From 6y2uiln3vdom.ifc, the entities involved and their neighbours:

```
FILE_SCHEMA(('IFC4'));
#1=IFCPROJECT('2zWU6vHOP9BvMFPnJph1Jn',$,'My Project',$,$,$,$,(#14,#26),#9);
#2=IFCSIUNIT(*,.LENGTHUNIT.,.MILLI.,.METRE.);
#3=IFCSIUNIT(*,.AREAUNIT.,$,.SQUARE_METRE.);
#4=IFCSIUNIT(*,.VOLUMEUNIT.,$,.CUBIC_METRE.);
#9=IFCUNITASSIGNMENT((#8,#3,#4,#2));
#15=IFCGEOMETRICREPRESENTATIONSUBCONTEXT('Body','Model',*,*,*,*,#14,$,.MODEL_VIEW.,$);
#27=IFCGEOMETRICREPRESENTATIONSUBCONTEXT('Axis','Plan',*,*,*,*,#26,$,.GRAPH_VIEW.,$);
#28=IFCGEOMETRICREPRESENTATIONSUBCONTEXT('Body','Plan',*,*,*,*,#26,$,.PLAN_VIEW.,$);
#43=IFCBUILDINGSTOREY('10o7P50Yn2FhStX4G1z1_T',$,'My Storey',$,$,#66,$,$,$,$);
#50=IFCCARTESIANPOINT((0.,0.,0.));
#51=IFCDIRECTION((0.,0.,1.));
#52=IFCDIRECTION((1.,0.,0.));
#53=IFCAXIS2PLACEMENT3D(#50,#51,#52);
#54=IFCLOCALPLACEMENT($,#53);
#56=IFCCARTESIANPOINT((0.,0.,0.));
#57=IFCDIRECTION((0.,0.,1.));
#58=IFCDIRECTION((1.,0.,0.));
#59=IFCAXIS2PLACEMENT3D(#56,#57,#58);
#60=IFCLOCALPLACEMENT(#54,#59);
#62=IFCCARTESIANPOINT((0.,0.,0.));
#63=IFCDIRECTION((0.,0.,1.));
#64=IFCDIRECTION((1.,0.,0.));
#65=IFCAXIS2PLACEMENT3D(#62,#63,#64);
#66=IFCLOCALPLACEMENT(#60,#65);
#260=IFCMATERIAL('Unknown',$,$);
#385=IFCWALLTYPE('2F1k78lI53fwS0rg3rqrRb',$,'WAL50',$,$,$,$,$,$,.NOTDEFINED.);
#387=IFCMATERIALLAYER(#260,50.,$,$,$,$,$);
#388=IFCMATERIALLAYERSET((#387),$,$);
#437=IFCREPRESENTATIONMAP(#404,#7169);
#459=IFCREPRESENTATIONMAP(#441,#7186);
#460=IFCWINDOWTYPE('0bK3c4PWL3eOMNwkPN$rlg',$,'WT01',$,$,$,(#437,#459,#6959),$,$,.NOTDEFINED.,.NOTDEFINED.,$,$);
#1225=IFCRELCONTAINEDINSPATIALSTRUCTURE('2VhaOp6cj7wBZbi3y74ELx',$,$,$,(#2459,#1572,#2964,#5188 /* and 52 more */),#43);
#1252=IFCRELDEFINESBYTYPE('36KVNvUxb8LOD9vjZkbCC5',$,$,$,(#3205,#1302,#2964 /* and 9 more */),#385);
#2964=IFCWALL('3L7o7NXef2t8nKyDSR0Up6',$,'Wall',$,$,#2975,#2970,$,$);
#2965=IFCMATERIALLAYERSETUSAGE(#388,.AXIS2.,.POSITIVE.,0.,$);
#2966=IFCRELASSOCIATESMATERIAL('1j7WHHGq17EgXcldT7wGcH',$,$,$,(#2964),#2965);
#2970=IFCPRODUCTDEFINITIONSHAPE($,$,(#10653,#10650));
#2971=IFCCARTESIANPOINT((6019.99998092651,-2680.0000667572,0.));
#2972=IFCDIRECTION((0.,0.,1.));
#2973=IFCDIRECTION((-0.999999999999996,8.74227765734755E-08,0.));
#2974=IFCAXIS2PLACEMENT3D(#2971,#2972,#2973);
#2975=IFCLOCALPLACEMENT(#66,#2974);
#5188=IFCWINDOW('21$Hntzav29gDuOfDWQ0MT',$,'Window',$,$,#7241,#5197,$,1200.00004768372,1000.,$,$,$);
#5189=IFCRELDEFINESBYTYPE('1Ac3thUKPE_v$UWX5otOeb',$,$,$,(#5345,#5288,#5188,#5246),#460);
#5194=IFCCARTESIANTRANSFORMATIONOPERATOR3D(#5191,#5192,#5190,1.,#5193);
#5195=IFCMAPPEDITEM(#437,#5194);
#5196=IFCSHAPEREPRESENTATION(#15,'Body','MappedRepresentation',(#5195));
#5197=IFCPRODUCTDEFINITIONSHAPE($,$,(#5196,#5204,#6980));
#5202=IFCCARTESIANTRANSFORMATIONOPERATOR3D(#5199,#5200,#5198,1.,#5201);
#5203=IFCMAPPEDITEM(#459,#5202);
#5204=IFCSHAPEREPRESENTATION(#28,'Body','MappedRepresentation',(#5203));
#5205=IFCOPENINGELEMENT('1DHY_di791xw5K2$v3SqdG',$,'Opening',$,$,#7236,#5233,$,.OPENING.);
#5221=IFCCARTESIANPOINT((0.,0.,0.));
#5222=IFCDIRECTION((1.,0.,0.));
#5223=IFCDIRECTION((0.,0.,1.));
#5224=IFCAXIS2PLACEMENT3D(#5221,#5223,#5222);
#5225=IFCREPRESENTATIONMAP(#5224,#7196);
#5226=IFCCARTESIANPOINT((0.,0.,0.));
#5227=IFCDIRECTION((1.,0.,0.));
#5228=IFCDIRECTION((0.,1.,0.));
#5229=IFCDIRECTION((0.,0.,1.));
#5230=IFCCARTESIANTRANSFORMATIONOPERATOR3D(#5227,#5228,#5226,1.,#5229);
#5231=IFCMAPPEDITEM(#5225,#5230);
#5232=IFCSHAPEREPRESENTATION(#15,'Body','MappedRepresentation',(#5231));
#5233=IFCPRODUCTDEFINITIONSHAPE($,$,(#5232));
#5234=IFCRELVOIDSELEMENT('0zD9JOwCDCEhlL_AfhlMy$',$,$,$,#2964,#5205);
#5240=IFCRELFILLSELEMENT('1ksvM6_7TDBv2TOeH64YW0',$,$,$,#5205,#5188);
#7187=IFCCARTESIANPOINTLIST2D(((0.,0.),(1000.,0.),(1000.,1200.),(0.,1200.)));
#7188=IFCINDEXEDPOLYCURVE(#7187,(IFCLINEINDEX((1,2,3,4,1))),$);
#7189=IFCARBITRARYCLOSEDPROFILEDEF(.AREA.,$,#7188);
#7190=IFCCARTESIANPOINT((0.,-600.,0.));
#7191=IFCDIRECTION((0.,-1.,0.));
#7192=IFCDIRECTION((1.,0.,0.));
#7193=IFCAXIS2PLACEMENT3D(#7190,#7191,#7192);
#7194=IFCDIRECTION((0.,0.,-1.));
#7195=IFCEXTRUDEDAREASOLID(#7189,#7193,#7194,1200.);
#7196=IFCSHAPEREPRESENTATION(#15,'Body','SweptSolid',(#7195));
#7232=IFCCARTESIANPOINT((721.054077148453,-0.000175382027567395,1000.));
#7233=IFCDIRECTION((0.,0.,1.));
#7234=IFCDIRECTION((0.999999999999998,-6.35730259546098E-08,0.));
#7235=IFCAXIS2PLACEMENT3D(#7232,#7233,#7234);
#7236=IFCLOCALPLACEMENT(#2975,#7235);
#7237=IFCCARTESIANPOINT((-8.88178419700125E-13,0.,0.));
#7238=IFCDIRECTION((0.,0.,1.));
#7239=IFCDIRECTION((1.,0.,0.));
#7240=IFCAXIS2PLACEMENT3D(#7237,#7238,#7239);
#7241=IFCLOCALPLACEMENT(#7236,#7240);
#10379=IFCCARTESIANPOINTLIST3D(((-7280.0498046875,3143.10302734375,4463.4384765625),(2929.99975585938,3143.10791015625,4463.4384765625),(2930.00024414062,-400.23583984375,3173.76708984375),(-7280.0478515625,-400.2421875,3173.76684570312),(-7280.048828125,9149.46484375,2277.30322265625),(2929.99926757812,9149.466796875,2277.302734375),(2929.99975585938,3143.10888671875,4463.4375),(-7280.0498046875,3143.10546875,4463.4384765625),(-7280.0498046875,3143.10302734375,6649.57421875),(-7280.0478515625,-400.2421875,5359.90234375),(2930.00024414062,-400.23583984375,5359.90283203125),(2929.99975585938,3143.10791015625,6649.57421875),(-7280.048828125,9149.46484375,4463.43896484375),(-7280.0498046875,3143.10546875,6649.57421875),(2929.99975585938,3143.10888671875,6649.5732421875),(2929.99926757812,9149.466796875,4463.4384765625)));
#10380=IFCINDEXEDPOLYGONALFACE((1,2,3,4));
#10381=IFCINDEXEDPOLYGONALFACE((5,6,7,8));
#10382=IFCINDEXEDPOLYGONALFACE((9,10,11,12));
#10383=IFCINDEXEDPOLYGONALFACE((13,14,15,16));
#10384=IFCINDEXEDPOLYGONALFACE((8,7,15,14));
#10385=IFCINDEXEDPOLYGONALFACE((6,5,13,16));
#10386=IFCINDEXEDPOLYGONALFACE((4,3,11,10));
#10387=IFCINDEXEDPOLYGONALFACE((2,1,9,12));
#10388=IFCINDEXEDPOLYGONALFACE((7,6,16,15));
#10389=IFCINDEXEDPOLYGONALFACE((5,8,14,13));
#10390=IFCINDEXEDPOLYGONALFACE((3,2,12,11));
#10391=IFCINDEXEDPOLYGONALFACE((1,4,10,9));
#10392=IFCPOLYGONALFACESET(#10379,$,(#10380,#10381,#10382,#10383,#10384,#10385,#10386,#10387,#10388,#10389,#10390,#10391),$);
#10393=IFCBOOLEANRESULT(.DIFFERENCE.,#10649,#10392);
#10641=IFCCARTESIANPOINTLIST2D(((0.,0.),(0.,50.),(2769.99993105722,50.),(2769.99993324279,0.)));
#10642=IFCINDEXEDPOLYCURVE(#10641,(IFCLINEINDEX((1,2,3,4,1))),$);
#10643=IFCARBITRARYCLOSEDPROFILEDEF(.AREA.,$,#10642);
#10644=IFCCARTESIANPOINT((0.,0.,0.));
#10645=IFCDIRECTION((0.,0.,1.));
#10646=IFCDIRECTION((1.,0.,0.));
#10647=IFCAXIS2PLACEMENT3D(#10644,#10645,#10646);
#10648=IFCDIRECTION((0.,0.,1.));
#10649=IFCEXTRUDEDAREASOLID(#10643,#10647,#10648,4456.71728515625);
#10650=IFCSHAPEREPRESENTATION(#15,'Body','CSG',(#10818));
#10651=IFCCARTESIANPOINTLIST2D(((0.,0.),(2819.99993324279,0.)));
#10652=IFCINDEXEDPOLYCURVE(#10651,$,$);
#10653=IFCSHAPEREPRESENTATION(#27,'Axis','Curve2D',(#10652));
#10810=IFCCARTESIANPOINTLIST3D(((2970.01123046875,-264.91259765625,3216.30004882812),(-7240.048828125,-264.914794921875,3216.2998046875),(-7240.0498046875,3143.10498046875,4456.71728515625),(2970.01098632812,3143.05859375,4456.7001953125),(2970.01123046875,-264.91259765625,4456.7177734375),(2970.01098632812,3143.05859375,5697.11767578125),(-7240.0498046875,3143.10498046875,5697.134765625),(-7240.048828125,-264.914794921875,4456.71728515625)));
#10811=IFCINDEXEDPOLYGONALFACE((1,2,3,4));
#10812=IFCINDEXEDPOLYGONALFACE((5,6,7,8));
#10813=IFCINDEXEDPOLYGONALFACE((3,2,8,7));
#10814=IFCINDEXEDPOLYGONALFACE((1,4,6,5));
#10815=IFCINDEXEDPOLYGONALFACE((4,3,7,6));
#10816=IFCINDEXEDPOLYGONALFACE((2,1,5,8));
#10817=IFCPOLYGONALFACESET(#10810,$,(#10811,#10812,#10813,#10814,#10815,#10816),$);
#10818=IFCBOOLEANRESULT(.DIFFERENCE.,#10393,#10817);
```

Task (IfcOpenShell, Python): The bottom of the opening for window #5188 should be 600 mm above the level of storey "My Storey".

```python
import numpy as np
import ifcopenshell
import ifcopenshell.api.geometry
import ifcopenshell.geom
import ifcopenshell.util.element
import ifcopenshell.util.placement
import ifcopenshell.util.shape
import ifcopenshell.util.unit

model = ifcopenshell.open("6y2uiln3vdom.ifc")
unit_scale = ifcopenshell.util.unit.calculate_unit_scale(model)

window = model.by_id(5188)
opening = window.FillsVoids[0].RelatingOpeningElement
storey = ifcopenshell.util.element.get_container(window, ifc_class="IfcBuildingStorey")
level = ifcopenshell.util.placement.get_local_placement(storey.ObjectPlacement)[2, 3]

# The opening's origin need not be at the sill, so measure its lowest point.
shape = ifcopenshell.geom.create_shape(ifcopenshell.geom.settings(), opening)
bottom = ifcopenshell.util.shape.get_shape_bottom_elevation(shape, shape.geometry) / unit_scale
dz = level + 0.6 / unit_scale - bottom

shift = np.array([0.0, 0.0, dz])
# The window is placed relative to its opening, so it follows when the opening moves.
matrix = ifcopenshell.util.placement.get_local_placement(opening.ObjectPlacement)
matrix[:3, 3] += shift
ifcopenshell.api.geometry.edit_object_placement(
    model, product=opening, matrix=matrix, is_si=False, should_transform_children=True
)

print(f"moved by {dz * unit_scale:+.3f} m")

model.write("6y2uiln3vdom-out.ifc")
```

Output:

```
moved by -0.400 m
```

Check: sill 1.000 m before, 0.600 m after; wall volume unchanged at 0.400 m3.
